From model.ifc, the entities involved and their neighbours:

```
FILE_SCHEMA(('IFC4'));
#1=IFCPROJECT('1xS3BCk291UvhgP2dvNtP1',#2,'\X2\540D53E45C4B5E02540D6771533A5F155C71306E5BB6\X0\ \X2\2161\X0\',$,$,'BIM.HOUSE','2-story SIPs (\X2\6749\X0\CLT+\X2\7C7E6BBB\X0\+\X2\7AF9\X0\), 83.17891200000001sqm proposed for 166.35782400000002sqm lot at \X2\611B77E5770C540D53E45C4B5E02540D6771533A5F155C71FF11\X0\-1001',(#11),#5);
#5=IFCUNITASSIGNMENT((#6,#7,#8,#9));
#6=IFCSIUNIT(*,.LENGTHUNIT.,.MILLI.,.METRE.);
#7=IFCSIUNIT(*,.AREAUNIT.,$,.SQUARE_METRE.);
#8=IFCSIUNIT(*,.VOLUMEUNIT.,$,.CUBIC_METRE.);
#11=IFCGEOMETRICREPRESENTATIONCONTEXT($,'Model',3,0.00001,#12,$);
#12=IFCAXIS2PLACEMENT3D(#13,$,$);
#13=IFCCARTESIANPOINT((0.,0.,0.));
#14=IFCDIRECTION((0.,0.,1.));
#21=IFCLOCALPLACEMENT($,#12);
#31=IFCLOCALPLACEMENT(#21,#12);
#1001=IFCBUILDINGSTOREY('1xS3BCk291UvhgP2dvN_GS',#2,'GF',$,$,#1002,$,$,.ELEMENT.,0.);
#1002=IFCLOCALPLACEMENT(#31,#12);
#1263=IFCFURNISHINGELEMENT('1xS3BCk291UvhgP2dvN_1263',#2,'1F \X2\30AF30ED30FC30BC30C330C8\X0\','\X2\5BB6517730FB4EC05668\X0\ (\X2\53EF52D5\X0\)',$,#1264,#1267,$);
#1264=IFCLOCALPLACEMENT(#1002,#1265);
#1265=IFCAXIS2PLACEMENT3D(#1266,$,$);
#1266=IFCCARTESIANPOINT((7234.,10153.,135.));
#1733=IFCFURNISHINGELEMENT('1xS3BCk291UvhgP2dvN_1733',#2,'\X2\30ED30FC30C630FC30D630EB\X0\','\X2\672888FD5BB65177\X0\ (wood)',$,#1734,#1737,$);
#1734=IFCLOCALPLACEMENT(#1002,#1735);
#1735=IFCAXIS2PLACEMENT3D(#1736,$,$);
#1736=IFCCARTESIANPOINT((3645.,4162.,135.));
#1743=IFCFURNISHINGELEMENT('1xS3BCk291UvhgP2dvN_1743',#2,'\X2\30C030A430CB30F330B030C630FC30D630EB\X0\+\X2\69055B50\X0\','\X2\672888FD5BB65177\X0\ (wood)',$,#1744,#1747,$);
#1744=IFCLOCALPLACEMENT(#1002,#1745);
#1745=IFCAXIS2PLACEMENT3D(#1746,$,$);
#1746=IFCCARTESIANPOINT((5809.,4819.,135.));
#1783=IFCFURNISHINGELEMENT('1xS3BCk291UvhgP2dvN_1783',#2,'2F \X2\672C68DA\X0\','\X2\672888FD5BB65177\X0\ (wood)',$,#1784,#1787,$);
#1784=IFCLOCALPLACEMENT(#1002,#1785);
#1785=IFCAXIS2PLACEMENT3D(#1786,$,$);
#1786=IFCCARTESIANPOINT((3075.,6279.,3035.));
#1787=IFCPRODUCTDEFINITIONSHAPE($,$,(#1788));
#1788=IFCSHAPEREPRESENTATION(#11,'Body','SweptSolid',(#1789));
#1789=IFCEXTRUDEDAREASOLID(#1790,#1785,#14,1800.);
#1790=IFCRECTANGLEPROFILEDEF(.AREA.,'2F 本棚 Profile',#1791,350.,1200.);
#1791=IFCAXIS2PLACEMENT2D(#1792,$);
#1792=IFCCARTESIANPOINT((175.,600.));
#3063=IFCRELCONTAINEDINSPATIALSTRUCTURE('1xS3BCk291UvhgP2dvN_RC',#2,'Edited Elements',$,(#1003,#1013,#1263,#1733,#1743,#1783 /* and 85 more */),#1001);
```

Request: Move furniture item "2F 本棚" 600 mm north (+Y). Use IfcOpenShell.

```python
import ifcopenshell
import ifcopenshell.api.geometry
import ifcopenshell.util.placement

model = ifcopenshell.open("model.ifc")

item = model.by_guid("1xS3BCk291UvhgP2dvN_1783")
matrix = ifcopenshell.util.placement.get_local_placement(item.ObjectPlacement)
matrix[1, 3] += 600.0
ifcopenshell.api.geometry.edit_object_placement(model, product=item, matrix=matrix, is_si=False)

print(ifcopenshell.util.placement.get_local_placement(item.ObjectPlacement).round(3) + 0.0)

model.write("model_v2.ifc")
```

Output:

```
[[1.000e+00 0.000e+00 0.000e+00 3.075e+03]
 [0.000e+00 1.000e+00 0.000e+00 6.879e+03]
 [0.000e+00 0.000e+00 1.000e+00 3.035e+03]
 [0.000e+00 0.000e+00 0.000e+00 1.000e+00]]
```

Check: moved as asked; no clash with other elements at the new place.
